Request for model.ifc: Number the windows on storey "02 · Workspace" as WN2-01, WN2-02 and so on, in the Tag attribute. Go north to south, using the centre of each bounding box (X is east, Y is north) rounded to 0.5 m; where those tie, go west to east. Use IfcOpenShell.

First a look at what the model holds.

```python
import ifcopenshell
import ifcopenshell.util.element
import ifcopenshell.util.placement

model = ifcopenshell.open("model.ifc")
print(model.schema)
storey = next(s for s in model.by_type("IfcBuildingStorey") if s.Name == "02 · Workspace")
windows = [e for e in ifcopenshell.util.element.get_decomposition(storey) if e.is_a("IfcWindow")]
for e in sorted(windows, key=lambda e: e.id()):
    origin = ifcopenshell.util.placement.get_local_placement(e.ObjectPlacement)[:3, 3]
    print(e.id(), e.Tag, e.Name, origin.round(2) + 0.0, sep=" | ")
```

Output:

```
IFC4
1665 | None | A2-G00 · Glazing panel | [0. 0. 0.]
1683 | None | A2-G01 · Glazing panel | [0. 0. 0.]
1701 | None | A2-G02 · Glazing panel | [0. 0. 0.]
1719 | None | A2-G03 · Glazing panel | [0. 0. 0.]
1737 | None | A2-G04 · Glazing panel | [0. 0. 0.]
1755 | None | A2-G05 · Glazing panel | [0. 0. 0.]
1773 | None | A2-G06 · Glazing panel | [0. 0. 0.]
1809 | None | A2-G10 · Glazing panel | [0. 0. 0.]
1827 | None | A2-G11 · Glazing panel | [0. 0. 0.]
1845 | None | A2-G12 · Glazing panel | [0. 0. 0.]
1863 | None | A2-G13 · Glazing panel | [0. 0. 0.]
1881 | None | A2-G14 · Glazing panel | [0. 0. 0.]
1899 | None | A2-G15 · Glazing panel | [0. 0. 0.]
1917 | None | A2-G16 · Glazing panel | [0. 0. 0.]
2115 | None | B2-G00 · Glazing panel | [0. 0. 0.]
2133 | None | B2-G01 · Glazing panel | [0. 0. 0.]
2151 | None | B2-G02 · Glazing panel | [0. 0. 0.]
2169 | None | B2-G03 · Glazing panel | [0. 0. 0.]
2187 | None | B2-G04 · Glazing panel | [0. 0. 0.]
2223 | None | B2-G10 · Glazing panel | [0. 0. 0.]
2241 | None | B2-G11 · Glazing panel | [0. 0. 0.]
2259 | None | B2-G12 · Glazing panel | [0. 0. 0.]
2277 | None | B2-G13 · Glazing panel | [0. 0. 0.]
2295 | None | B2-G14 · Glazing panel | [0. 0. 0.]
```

```python
import ifcopenshell
import ifcopenshell.geom
import ifcopenshell.util.element
import ifcopenshell.util.shape

model = ifcopenshell.open("model.ifc")
settings = ifcopenshell.geom.settings()
settings.set("use-world-coords", True)


def centre(element):
    shape = ifcopenshell.geom.create_shape(settings, element)
    return ifcopenshell.util.shape.get_bbox_centroid(shape.geometry)


storey = next(s for s in model.by_type("IfcBuildingStorey") if s.Name == "02 · Workspace")
windows = [e for e in ifcopenshell.util.element.get_decomposition(storey) if e.is_a("IfcWindow")]

# Insertion points can sit at a corner or the storey origin, so sort by the geometry (in metres).
centres = {e: centre(e) for e in windows}
windows.sort(key=lambda e: (-round(centres[e][1] / 0.5), centres[e][0]))

for i, e in enumerate(windows, start=1):
    number = f"WN2-{i:02d}"
    e.Tag = number
    print(e.id(), number)

model.write("model_v2.ifc")
```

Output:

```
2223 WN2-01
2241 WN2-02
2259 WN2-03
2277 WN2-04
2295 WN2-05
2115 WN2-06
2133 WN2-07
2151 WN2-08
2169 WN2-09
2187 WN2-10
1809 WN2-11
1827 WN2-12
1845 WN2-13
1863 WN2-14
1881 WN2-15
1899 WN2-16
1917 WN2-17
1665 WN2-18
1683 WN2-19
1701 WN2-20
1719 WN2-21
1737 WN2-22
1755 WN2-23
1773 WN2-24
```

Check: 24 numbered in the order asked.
